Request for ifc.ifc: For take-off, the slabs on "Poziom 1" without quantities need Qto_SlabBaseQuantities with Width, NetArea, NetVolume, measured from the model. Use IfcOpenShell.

First a look at what the model holds.

```python
import ifcopenshell
import ifcopenshell.util.element
import ifcopenshell.util.unit

model = ifcopenshell.open("ifc.ifc")
print(model.schema)
for unit_type in ("LENGTHUNIT", "AREAUNIT", "VOLUMEUNIT"):
    print(unit_type, ifcopenshell.util.unit.calculate_unit_scale(model, unit_type))
storey = next(s for s in model.by_type("IfcBuildingStorey") if s.Name == "Poziom 1")
slabs = [e for e in ifcopenshell.util.element.get_decomposition(storey) if e.is_a("IfcSlab")]
for e in sorted(slabs, key=lambda e: e.id()):
    print(e.id(), e.is_a(), e.Name, list(ifcopenshell.util.element.get_psets(e, qtos_only=True)), sep=" | ")
```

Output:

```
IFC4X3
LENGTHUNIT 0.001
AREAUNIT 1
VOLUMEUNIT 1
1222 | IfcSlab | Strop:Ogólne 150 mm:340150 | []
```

```python
import ifcopenshell
import ifcopenshell.api.pset
import ifcopenshell.geom
import ifcopenshell.util.element
import ifcopenshell.util.shape
import ifcopenshell.util.unit

model = ifcopenshell.open("ifc.ifc")
unit_scale = ifcopenshell.util.unit.calculate_unit_scale(model)
area_scale = ifcopenshell.util.unit.calculate_unit_scale(model, "AREAUNIT")
volume_scale = ifcopenshell.util.unit.calculate_unit_scale(model, "VOLUMEUNIT")
settings = ifcopenshell.geom.settings()

storey = next(s for s in model.by_type("IfcBuildingStorey") if s.Name == "Poziom 1")
slabs = [e for e in ifcopenshell.util.element.get_decomposition(storey) if e.is_a("IfcSlab")]

for e in sorted(slabs, key=lambda e: e.id()):
    if ifcopenshell.util.element.get_psets(e, qtos_only=True, should_inherit=False):
        continue
    # Geometry comes back in metres, in the element's own axes.
    shape = ifcopenshell.geom.create_shape(settings, e)
    values = {
        "Width": ifcopenshell.util.shape.get_z(shape.geometry) / unit_scale,
        "NetArea": ifcopenshell.util.shape.get_footprint_area(shape.geometry) / area_scale,
        "NetVolume": ifcopenshell.util.shape.get_volume(shape.geometry) / volume_scale,
    }
    qto = ifcopenshell.api.pset.add_qto(model, product=e, name="Qto_SlabBaseQuantities")
    ifcopenshell.api.pset.edit_qto(model, qto=qto, properties=values)
    print(e.id(), {k: round(v, 3) for k, v in values.items()})

model.write("ifc_edited.ifc")
```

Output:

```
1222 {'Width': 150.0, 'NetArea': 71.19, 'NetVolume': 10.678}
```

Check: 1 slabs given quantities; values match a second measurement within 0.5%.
